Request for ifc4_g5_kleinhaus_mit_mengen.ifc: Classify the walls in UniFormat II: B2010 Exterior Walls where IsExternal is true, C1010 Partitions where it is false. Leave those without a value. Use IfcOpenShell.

First a look at what the model holds.

```python
import ifcopenshell
import ifcopenshell.util.element

model = ifcopenshell.open("ifc4_g5_kleinhaus_mit_mengen.ifc")
print(model.schema)
print("classifications:", [c.Name for c in model.by_type("IfcClassification")])
values = [ifcopenshell.util.element.get_pset(e, "Pset_WallCommon", "IsExternal") for e in model.by_type("IfcWall")]
for value in (True, False, None):
    print("IsExternal", value, values.count(value))
```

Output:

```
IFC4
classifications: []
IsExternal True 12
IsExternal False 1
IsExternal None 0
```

```python
import ifcopenshell
import ifcopenshell.api.classification
import ifcopenshell.util.element

model = ifcopenshell.open("ifc4_g5_kleinhaus_mit_mengen.ifc")

system = ifcopenshell.api.classification.add_classification(model, classification="UniFormat II")

walls = model.by_type("IfcWall")
external = {e: ifcopenshell.util.element.get_pset(e, "Pset_WallCommon", "IsExternal") for e in walls}
for flag, code, name in ((True, "B2010", "Exterior Walls"), (False, "C1010", "Partitions")):
    products = [e for e in walls if external[e] is flag]
    ifcopenshell.api.classification.add_reference(
        model, products=products, classification=system, identification=code, name=name
    )
    print(code, len(products))

model.write("ifc4_g5_kleinhaus_mit_mengen_updated.ifc")
```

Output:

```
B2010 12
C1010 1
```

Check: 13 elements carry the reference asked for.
